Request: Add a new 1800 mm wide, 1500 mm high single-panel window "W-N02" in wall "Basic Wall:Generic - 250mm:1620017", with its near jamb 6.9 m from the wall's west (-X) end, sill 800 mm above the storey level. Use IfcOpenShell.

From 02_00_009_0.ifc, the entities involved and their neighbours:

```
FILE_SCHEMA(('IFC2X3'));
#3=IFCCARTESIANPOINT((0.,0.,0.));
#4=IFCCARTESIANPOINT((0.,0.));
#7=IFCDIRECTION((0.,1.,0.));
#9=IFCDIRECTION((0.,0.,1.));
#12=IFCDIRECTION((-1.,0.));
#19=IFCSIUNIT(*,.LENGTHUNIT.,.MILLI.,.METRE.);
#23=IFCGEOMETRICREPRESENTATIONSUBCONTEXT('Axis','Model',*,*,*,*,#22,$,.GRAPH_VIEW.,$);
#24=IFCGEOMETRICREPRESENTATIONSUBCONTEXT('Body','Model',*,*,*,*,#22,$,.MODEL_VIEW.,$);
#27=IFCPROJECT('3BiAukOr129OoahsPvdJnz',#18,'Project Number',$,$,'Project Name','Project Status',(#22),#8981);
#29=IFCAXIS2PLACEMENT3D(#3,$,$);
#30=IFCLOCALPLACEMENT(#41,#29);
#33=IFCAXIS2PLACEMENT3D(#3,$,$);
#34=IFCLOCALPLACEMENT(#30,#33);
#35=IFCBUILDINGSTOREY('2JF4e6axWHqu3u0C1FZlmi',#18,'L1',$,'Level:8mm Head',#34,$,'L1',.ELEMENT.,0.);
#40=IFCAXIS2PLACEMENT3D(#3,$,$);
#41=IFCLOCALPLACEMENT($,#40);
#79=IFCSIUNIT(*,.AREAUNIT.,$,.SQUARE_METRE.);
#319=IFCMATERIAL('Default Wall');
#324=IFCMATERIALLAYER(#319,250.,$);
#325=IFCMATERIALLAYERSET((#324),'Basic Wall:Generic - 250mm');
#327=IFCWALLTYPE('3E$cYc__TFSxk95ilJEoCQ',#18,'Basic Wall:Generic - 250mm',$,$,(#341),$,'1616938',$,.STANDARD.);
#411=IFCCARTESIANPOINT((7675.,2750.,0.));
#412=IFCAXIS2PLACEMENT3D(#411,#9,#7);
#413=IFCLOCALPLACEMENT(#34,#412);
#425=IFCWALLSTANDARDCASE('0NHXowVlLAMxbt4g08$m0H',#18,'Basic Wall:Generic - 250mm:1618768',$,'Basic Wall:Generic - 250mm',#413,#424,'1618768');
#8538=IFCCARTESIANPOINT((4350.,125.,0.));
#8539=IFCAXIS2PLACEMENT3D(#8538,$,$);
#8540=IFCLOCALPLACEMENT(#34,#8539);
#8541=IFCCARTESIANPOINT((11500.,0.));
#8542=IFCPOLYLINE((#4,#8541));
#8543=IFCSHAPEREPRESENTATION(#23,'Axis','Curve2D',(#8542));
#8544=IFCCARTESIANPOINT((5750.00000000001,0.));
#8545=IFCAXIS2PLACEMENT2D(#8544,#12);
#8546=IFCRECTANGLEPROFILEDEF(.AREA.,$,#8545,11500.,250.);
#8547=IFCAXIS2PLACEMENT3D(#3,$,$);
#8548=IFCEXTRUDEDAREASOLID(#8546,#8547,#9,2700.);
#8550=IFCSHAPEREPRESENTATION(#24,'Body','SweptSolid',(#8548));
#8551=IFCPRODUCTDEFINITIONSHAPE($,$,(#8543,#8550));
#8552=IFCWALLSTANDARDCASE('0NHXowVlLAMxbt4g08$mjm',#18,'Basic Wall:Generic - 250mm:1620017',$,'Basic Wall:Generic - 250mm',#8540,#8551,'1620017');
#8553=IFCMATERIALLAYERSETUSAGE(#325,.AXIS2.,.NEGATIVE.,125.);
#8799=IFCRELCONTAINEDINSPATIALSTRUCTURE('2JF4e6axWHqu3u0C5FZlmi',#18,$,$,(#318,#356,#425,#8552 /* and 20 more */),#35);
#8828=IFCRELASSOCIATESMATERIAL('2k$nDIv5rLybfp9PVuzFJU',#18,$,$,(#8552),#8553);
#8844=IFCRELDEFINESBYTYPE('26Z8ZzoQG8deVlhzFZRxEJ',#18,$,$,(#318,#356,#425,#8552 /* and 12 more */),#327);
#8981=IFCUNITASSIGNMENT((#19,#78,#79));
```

```python
import numpy as np
import ifcopenshell
import ifcopenshell.api.feature
import ifcopenshell.api.geometry
import ifcopenshell.api.root
import ifcopenshell.api.spatial
import ifcopenshell.api.type
import ifcopenshell.geom
import ifcopenshell.util.element
import ifcopenshell.util.placement
import ifcopenshell.util.representation
import ifcopenshell.util.shape
import ifcopenshell.util.unit

model = ifcopenshell.open("02_00_009_0.ifc")
unit_scale = ifcopenshell.util.unit.calculate_unit_scale(model)
settings = ifcopenshell.geom.settings()


def volume(element):
    """Net volume in cubic metres, openings subtracted."""
    shape = ifcopenshell.geom.create_shape(settings, element)
    return ifcopenshell.util.shape.get_volume(shape.geometry)


wall = model.by_id(8552)
storey = ifcopenshell.util.element.get_container(wall, ifc_class="IfcBuildingStorey")
context = ifcopenshell.util.representation.get_context(model, "Model", "Body", "MODEL_VIEW")
before = volume(wall)

width, height, from_end, sill = 1.8, 1.5, 6.9, 0.8  # metres

# The wall runs along its own X axis, and the end named is its -X end.
wall_shape = ifcopenshell.geom.create_shape(settings, wall)
x, y, z = ifcopenshell.util.shape.get_vertices(wall_shape.geometry).T
start = x.min() + from_end
face, thickness = float(y.min()), float(y.max() - y.min())
wall_matrix = ifcopenshell.util.placement.get_local_placement(wall.ObjectPlacement)
level = ifcopenshell.util.placement.get_local_placement(storey.ObjectPlacement)[2, 3]


def in_wall(x, y):
    """Placement at x, y metres in the wall's axes, at sill height."""
    matrix = wall_matrix.copy()
    matrix[:, 3] = wall_matrix @ np.array([x / unit_scale, y / unit_scale, 0.0, 1.0])
    matrix[2, 3] = level + sill / unit_scale
    return matrix


# Opening: a box that overshoots both wall faces by 50 mm.
opening = ifcopenshell.api.root.create_entity(model, ifc_class="IfcOpeningElement")
box = ifcopenshell.api.geometry.add_wall_representation(
    model, context=context, length=width, height=height, thickness=thickness + 0.1
)
ifcopenshell.api.geometry.assign_representation(model, product=opening, representation=box)
ifcopenshell.api.geometry.edit_object_placement(model, product=opening, matrix=in_wall(start, face - 0.05), is_si=False)
ifcopenshell.api.feature.add_feature(model, feature=opening, element=wall)

window = ifcopenshell.api.root.create_entity(model, ifc_class="IfcWindow", name="W-N02")
window.OverallWidth, window.OverallHeight = width / unit_scale, height / unit_scale
body = ifcopenshell.api.geometry.add_window_representation(
    model,
    context=context,
    overall_width=window.OverallWidth,
    overall_height=window.OverallHeight,
    partition_type="SINGLE_PANEL",
)
ifcopenshell.api.geometry.assign_representation(model, product=window, representation=body)
ifcopenshell.api.spatial.assign_container(model, products=[window], relating_structure=storey)
fills = ifcopenshell.api.feature.add_filling(model, opening=opening, element=window)
fills.OwnerHistory = window.OwnerHistory  # required in IFC2X3

# IFC2X3 keeps the operation on the window style.
style = ifcopenshell.api.root.create_entity(model, ifc_class="IfcWindowStyle", name="W-N02")
style.OperationType, style.ConstructionType = "SINGLE_PANEL", "NOTDEFINED"
style.ParameterTakesPrecedence = style.Sizeable = False
ifcopenshell.api.type.assign_type(model, related_objects=[window], relating_type=style)

# Centre the window in the wall's thickness.
ifcopenshell.api.geometry.edit_object_placement(model, product=window, matrix=in_wall(start, face), is_si=False)
window_shape = ifcopenshell.geom.create_shape(settings, window)
depth = ifcopenshell.util.shape.get_vertices(window_shape.geometry)[:, 1]
offset = face + thickness / 2 - (depth.min() + depth.max()) / 2
ifcopenshell.api.geometry.edit_object_placement(model, product=window, matrix=in_wall(start, offset), is_si=False)

after = volume(wall)

print(f"wall volume {before:.3f} -> {after:.3f} m3")

model.write("02_00_009_0_rev.ifc")
```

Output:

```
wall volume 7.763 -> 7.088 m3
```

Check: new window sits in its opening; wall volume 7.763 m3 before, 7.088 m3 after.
